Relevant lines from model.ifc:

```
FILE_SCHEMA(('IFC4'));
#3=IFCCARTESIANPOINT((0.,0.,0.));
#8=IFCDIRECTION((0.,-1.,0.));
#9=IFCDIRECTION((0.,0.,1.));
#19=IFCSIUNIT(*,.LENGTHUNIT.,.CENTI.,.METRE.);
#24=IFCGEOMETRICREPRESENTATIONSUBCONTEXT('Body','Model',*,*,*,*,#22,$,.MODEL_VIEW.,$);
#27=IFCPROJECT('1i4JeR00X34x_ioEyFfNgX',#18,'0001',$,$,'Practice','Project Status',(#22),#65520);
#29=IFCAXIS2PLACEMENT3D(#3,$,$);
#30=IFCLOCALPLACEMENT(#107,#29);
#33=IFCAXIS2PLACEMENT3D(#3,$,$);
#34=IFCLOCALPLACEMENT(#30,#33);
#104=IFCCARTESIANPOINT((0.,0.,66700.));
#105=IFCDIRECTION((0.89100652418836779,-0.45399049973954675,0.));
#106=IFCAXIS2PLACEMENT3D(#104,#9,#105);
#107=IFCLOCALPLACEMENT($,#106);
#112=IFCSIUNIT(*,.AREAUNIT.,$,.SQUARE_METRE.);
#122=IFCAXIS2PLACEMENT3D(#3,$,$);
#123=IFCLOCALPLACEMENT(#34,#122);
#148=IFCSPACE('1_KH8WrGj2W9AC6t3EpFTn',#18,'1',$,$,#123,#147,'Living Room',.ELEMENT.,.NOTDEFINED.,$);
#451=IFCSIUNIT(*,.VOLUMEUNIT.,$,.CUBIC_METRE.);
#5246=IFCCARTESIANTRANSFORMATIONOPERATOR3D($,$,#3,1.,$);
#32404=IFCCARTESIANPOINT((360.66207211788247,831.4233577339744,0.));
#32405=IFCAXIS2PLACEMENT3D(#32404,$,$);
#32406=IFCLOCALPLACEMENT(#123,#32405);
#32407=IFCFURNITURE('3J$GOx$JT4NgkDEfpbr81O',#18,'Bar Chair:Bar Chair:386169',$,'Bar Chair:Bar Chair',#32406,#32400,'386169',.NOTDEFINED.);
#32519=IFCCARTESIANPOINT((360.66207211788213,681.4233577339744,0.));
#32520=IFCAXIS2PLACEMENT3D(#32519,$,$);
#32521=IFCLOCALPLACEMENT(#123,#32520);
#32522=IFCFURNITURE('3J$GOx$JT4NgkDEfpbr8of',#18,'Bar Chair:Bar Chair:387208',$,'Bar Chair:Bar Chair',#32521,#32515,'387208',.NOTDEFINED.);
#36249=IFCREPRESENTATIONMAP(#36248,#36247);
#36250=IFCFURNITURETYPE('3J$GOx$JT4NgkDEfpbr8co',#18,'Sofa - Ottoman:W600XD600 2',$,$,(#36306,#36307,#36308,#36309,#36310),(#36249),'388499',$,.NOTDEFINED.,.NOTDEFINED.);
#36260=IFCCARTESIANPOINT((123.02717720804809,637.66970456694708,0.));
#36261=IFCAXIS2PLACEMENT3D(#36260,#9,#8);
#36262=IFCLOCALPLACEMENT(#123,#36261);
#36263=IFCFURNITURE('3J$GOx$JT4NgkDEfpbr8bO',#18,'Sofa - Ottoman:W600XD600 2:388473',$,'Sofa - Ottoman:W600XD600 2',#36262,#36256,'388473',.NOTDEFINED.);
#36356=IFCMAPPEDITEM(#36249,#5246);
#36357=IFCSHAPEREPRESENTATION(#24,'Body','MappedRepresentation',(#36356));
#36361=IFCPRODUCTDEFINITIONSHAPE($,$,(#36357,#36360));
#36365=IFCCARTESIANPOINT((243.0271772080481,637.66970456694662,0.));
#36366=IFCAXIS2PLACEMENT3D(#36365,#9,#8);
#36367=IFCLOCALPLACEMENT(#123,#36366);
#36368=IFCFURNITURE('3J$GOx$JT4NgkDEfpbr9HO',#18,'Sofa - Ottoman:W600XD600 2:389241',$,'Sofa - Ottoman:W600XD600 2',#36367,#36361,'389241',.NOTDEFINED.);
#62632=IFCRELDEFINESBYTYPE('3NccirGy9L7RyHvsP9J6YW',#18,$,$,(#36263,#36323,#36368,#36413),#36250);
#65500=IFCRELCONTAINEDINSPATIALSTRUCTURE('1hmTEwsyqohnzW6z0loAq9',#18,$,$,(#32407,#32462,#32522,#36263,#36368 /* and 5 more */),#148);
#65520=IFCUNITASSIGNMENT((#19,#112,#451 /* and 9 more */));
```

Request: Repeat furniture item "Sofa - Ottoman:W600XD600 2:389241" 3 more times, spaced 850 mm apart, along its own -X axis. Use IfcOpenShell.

```python
import ifcopenshell
import ifcopenshell.api.geometry
import ifcopenshell.api.root
import ifcopenshell.util.element
import ifcopenshell.util.placement
import ifcopenshell.util.unit

model = ifcopenshell.open("model.ifc")
unit_scale = ifcopenshell.util.unit.calculate_unit_scale(model)


def reuse_history(source, copy):
    """copy_class also copies each property set's owner history, people and application; keep the originals."""
    for rel in copy.IsDefinedBy:
        if rel.is_a("IfcRelDefinesByProperties") and (history := rel.RelatingPropertyDefinition.OwnerHistory):
            rel.RelatingPropertyDefinition.OwnerHistory = source.OwnerHistory
            ifcopenshell.util.element.remove_deep2(model, history)


source = model.by_guid("3J$GOx$JT4NgkDEfpbr9HO")
base = ifcopenshell.util.placement.get_local_placement(source.ObjectPlacement)
step = -base[:3, 0] * 0.85 / unit_scale

for i in range(1, 4):
    copy = ifcopenshell.api.root.copy_class(model, product=source)
    copy.Representation = ifcopenshell.util.element.copy_deep(
        model, source.Representation, exclude=["IfcGeometricRepresentationContext", "IfcRepresentationMap"]
    )
    copy.Name = "Sofa - Ottoman:W600XD600 2"
    copy.Tag = None
    reuse_history(source, copy)
    matrix = base.copy()
    matrix[:3, 3] += i * step
    print("added at", matrix[:3, 3].round(3) + 0.0)
    ifcopenshell.api.geometry.edit_object_placement(model, product=copy, matrix=matrix, is_si=False)

model.write("model_edited.ifc")
```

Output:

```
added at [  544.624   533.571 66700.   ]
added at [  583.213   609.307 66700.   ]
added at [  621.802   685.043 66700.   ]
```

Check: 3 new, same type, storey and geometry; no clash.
